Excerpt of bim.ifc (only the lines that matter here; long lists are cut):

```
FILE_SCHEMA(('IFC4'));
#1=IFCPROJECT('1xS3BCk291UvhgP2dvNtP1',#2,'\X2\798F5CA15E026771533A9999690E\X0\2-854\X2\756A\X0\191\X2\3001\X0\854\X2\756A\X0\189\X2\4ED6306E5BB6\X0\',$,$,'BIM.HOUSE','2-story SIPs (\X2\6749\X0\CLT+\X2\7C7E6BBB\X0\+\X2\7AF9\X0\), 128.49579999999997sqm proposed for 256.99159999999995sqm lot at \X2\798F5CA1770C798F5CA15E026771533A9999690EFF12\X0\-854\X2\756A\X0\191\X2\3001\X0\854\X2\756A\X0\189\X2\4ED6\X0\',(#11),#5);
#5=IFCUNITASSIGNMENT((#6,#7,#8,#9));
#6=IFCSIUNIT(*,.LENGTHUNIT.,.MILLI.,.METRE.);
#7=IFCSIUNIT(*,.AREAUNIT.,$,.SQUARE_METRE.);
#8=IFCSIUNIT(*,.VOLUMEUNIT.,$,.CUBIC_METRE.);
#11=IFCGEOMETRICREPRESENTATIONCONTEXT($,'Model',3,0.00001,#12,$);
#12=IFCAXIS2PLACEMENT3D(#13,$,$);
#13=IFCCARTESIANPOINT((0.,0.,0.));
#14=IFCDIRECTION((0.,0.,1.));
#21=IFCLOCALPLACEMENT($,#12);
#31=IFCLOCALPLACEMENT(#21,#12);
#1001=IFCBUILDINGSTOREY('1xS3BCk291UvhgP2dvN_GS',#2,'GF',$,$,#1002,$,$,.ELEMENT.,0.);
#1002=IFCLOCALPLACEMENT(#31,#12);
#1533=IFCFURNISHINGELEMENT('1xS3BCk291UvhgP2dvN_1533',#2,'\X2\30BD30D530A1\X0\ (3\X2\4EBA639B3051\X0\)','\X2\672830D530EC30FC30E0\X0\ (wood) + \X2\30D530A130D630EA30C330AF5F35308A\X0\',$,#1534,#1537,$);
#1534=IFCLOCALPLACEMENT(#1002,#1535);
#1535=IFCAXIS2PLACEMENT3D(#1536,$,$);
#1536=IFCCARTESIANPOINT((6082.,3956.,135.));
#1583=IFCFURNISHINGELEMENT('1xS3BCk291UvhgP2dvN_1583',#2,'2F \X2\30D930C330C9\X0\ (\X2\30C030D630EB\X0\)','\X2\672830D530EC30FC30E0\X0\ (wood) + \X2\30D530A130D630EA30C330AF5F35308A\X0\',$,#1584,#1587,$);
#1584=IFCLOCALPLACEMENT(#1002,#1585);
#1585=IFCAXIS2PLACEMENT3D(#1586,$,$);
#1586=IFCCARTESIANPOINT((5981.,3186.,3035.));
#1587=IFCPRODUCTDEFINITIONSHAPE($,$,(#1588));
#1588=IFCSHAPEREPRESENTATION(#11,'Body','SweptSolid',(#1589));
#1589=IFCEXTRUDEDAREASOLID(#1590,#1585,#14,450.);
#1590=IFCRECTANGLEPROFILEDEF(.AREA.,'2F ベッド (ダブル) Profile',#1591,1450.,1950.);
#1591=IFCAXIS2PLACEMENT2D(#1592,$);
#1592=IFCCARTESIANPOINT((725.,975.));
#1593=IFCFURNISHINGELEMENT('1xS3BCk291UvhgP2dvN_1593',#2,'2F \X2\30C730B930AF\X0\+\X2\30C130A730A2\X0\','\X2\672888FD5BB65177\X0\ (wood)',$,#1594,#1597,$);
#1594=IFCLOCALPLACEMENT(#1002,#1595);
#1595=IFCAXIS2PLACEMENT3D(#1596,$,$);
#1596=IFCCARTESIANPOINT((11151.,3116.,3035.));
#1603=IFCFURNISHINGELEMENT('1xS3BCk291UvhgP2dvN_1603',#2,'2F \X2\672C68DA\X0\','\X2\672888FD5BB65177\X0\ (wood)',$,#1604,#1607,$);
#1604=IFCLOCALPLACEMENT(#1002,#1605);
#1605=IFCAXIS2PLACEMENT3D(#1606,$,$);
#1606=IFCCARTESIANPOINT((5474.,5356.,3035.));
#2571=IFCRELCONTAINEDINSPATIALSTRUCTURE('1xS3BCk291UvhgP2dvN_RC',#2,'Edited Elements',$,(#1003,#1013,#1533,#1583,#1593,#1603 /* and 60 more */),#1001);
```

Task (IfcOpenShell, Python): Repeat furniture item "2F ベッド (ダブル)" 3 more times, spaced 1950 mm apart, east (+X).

```python
import numpy as np
import ifcopenshell
import ifcopenshell.api.geometry
import ifcopenshell.api.root
import ifcopenshell.util.element
import ifcopenshell.util.placement
import ifcopenshell.util.unit

model = ifcopenshell.open("bim.ifc")
unit_scale = ifcopenshell.util.unit.calculate_unit_scale(model)


def reuse_history(source, copy):
    """copy_class also copies each property set's owner history, people and application; keep the originals."""
    for rel in copy.IsDefinedBy:
        if rel.is_a("IfcRelDefinesByProperties") and (history := rel.RelatingPropertyDefinition.OwnerHistory):
            rel.RelatingPropertyDefinition.OwnerHistory = source.OwnerHistory
            ifcopenshell.util.element.remove_deep2(model, history)


source = model.by_guid("1xS3BCk291UvhgP2dvN_1583")
base = ifcopenshell.util.placement.get_local_placement(source.ObjectPlacement)
step = np.array([1.0, 0.0, 0.0]) * 1.95 / unit_scale

for i in range(1, 4):
    copy = ifcopenshell.api.root.copy_class(model, product=source)
    copy.Representation = ifcopenshell.util.element.copy_deep(
        model, source.Representation, exclude=["IfcGeometricRepresentationContext", "IfcRepresentationMap"]
    )
    reuse_history(source, copy)
    matrix = base.copy()
    matrix[:3, 3] += i * step
    print("added at", matrix[:3, 3].round(3) + 0.0)
    ifcopenshell.api.geometry.edit_object_placement(model, product=copy, matrix=matrix, is_si=False)

model.write("bim_edited.ifc")
```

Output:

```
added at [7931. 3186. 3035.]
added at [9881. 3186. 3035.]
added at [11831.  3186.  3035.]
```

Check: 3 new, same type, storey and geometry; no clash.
